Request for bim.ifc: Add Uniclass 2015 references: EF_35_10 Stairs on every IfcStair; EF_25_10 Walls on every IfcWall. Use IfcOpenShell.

First a look at what the model holds.

```python
import ifcopenshell

model = ifcopenshell.open("bim.ifc")
print(model.schema)
print("classifications:", [c.Name for c in model.by_type("IfcClassification")])
for ifc_class in ("IfcDoor", "IfcRoof", "IfcStair", "IfcWall", "IfcWindow"):
    print(ifc_class, len(model.by_type(ifc_class)))
```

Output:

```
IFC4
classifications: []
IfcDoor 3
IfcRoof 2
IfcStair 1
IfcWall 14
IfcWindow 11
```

```python
import ifcopenshell
import ifcopenshell.api.classification

model = ifcopenshell.open("bim.ifc")

system = ifcopenshell.api.classification.add_classification(model, classification="Uniclass 2015")

codes = {
    "IfcStair": ("EF_35_10", "Stairs"),
    "IfcWall": ("EF_25_10", "Walls"),
}
for ifc_class, (code, name) in codes.items():
    products = model.by_type(ifc_class)
    ifcopenshell.api.classification.add_reference(
        model, products=products, classification=system, identification=code, name=name
    )
    print(code, len(products))

model.write("bim_edited.ifc")
```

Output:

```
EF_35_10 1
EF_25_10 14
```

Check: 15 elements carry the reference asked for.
